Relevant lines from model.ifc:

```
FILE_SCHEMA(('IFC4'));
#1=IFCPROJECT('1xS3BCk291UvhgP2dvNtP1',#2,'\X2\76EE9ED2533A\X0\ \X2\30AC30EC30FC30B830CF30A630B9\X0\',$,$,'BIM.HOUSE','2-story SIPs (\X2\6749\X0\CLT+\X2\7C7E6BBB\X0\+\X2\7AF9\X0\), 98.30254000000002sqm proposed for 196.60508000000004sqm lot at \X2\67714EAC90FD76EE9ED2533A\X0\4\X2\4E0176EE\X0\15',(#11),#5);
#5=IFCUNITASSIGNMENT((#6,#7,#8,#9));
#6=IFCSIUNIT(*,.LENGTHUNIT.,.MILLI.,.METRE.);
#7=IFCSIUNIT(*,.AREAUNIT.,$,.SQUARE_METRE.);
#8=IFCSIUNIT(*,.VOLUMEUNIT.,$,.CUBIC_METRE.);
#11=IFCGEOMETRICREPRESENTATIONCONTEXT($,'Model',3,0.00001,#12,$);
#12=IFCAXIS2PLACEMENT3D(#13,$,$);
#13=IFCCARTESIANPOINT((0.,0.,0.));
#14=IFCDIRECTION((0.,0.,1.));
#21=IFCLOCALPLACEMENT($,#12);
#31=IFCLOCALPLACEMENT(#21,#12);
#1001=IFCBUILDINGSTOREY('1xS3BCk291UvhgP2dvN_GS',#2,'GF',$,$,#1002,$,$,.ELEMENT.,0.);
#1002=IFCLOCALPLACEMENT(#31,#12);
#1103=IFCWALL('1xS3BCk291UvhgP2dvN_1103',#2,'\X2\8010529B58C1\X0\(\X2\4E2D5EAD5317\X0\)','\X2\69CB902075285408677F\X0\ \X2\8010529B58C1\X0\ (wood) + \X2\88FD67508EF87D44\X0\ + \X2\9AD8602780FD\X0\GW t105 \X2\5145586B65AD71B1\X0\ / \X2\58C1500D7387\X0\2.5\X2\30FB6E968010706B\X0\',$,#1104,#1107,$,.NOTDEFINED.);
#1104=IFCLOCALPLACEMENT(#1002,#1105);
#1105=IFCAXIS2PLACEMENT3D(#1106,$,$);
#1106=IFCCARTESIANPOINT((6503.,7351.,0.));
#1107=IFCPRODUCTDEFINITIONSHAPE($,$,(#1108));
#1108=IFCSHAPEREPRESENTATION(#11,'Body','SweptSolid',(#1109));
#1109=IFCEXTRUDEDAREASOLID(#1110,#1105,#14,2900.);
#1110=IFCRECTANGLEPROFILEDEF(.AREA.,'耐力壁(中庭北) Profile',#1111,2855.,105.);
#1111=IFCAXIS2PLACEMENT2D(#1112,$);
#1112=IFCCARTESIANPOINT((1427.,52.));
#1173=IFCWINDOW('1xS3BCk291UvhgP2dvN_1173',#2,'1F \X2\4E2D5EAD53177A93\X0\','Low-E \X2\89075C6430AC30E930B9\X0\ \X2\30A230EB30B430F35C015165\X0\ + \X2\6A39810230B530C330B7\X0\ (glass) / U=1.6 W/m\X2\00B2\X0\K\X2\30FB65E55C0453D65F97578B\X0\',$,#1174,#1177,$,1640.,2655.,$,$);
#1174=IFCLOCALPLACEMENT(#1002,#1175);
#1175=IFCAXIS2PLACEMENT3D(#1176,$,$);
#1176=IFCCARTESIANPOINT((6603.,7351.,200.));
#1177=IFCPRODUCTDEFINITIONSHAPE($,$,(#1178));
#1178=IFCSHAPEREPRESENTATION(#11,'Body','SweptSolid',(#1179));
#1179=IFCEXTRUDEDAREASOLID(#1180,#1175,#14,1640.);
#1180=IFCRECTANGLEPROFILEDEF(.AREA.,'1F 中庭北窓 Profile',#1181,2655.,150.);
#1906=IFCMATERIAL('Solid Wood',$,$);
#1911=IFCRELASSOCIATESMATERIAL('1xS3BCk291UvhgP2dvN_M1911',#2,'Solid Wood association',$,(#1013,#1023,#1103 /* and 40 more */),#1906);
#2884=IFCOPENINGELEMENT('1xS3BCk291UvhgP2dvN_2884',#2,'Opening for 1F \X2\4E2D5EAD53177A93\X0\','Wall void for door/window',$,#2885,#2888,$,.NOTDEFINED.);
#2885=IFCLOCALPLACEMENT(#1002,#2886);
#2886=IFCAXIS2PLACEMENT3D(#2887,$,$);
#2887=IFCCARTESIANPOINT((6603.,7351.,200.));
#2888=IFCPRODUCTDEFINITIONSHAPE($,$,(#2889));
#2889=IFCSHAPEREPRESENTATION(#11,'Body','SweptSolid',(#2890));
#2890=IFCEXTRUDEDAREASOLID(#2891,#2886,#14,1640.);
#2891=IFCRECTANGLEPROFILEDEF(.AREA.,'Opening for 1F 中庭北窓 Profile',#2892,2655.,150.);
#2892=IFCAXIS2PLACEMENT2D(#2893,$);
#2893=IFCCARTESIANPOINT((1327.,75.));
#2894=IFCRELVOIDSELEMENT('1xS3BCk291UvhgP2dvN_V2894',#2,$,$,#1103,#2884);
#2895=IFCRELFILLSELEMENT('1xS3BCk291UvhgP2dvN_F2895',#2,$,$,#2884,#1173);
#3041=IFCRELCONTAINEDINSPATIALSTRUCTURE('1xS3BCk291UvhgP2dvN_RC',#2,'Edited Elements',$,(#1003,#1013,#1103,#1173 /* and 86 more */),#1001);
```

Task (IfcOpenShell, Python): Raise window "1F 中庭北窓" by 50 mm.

```python
import numpy as np
import ifcopenshell
import ifcopenshell.api.geometry
import ifcopenshell.util.placement
import ifcopenshell.util.unit

model = ifcopenshell.open("model.ifc")
unit_scale = ifcopenshell.util.unit.calculate_unit_scale(model)

window = model.by_id(1173)
opening = window.FillsVoids[0].RelatingOpeningElement
dz = 50.0

shift = np.array([0.0, 0.0, dz])
# The window is not placed relative to its opening, so move both.
for product in (opening, window):
    matrix = ifcopenshell.util.placement.get_local_placement(product.ObjectPlacement)
    matrix[:3, 3] += shift
    ifcopenshell.api.geometry.edit_object_placement(model, product=product, matrix=matrix, is_si=False)

print(f"moved by {dz * unit_scale:+.3f} m")

model.write("model_rev.ifc")
```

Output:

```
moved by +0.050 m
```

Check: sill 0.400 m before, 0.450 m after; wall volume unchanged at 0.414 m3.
